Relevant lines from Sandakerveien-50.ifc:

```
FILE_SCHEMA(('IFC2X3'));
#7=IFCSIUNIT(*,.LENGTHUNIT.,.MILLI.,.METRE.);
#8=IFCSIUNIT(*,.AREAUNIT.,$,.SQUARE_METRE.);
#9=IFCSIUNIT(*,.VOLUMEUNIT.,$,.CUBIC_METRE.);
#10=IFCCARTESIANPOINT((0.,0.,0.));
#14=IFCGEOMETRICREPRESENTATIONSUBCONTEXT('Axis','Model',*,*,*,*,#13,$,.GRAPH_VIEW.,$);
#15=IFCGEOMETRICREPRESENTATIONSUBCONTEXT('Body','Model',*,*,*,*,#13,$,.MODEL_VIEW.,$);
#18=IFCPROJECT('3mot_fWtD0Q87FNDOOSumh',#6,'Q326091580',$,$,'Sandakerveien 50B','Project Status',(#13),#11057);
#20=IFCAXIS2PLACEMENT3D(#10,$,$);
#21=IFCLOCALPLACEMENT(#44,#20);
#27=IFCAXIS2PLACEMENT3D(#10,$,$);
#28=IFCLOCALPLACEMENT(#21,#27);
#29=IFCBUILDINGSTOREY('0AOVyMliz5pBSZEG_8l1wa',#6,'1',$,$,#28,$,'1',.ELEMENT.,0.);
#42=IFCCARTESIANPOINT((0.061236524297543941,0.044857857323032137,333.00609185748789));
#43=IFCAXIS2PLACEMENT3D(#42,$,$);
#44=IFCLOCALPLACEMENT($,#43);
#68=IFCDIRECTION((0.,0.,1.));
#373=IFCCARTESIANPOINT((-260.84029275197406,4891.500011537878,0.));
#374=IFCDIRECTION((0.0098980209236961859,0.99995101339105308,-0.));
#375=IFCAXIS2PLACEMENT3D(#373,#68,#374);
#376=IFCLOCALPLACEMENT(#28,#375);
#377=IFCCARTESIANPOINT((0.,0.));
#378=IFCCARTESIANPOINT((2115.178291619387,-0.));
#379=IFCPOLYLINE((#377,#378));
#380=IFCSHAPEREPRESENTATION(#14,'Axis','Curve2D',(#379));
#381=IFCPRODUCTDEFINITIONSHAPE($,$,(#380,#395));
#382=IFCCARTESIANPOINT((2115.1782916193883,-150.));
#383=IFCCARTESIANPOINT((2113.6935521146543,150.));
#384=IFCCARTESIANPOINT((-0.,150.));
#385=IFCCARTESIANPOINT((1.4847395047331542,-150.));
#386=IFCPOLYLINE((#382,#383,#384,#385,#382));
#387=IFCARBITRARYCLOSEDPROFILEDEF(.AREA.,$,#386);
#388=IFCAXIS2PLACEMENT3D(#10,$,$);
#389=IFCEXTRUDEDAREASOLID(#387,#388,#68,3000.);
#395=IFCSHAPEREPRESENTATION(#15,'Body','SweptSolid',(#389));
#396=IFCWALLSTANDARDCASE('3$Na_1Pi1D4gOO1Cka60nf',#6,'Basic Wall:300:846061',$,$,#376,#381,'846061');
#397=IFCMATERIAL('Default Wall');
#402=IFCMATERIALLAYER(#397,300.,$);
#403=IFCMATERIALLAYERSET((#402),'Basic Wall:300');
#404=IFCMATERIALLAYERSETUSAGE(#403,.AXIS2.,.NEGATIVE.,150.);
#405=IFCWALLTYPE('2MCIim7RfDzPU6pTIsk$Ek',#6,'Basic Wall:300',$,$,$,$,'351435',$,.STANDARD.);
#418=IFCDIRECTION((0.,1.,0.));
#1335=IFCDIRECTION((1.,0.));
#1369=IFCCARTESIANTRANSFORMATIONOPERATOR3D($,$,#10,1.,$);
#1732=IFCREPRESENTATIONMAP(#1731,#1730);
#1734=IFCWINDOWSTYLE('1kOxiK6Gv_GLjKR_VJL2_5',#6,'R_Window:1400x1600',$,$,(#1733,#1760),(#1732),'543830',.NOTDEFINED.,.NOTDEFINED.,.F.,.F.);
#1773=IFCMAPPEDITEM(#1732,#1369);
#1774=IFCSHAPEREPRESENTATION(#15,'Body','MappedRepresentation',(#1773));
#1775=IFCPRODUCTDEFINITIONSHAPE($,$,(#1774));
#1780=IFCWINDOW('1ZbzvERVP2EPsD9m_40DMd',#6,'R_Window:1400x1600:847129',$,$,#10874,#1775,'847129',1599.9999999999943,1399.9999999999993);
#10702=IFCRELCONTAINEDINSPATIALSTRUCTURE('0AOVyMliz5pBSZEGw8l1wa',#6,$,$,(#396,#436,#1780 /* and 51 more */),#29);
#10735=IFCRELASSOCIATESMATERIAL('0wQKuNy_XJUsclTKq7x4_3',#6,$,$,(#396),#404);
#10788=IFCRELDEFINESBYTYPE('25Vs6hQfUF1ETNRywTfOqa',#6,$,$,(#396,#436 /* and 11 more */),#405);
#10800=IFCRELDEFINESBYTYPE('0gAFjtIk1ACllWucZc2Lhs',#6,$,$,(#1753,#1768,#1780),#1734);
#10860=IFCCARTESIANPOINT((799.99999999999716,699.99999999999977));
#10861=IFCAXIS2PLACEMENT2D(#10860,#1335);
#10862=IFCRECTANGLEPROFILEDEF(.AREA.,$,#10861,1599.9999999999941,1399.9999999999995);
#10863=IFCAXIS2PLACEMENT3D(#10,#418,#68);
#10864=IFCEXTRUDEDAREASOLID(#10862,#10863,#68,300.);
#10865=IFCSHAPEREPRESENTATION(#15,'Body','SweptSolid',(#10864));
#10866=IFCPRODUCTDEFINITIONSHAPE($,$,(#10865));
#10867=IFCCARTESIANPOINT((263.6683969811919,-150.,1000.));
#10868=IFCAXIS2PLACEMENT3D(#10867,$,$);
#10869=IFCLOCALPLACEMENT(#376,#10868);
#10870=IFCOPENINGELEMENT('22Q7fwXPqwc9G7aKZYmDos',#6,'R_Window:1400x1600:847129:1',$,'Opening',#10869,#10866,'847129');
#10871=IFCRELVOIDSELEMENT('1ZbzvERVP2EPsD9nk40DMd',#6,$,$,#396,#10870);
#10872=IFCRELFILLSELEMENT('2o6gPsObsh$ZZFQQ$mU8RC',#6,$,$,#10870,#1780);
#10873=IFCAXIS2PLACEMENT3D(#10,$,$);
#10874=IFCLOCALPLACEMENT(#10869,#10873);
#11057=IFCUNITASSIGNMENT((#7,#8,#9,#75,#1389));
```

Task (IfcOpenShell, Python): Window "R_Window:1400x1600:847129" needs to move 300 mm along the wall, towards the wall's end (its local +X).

```python
import ifcopenshell
import ifcopenshell.api.geometry
import ifcopenshell.util.placement

model = ifcopenshell.open("Sandakerveien-50.ifc")

window = model.by_guid("1ZbzvERVP2EPsD9m_40DMd")
opening = window.FillsVoids[0].RelatingOpeningElement
wall = opening.VoidsElements[0].RelatingBuildingElement

wall_matrix = ifcopenshell.util.placement.get_local_placement(wall.ObjectPlacement)
shift = wall_matrix[:3, 0] * 300.0
before = ifcopenshell.util.placement.get_local_placement(window.ObjectPlacement)[:3, 3].copy()

# The window is placed relative to its opening, so it follows when the opening moves.
matrix = ifcopenshell.util.placement.get_local_placement(opening.ObjectPlacement)
matrix[:3, 3] += shift
ifcopenshell.api.geometry.edit_object_placement(
    model, product=opening, matrix=matrix, is_si=False, should_transform_children=True
)

after = ifcopenshell.util.placement.get_local_placement(window.ObjectPlacement)[:3, 3]
print("window moved by", (after - before).round(3) + 0.0)

model.write("Sandakerveien-50_rev.ifc")
```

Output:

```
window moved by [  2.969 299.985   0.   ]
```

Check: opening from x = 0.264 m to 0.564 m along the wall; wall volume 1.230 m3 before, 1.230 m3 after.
